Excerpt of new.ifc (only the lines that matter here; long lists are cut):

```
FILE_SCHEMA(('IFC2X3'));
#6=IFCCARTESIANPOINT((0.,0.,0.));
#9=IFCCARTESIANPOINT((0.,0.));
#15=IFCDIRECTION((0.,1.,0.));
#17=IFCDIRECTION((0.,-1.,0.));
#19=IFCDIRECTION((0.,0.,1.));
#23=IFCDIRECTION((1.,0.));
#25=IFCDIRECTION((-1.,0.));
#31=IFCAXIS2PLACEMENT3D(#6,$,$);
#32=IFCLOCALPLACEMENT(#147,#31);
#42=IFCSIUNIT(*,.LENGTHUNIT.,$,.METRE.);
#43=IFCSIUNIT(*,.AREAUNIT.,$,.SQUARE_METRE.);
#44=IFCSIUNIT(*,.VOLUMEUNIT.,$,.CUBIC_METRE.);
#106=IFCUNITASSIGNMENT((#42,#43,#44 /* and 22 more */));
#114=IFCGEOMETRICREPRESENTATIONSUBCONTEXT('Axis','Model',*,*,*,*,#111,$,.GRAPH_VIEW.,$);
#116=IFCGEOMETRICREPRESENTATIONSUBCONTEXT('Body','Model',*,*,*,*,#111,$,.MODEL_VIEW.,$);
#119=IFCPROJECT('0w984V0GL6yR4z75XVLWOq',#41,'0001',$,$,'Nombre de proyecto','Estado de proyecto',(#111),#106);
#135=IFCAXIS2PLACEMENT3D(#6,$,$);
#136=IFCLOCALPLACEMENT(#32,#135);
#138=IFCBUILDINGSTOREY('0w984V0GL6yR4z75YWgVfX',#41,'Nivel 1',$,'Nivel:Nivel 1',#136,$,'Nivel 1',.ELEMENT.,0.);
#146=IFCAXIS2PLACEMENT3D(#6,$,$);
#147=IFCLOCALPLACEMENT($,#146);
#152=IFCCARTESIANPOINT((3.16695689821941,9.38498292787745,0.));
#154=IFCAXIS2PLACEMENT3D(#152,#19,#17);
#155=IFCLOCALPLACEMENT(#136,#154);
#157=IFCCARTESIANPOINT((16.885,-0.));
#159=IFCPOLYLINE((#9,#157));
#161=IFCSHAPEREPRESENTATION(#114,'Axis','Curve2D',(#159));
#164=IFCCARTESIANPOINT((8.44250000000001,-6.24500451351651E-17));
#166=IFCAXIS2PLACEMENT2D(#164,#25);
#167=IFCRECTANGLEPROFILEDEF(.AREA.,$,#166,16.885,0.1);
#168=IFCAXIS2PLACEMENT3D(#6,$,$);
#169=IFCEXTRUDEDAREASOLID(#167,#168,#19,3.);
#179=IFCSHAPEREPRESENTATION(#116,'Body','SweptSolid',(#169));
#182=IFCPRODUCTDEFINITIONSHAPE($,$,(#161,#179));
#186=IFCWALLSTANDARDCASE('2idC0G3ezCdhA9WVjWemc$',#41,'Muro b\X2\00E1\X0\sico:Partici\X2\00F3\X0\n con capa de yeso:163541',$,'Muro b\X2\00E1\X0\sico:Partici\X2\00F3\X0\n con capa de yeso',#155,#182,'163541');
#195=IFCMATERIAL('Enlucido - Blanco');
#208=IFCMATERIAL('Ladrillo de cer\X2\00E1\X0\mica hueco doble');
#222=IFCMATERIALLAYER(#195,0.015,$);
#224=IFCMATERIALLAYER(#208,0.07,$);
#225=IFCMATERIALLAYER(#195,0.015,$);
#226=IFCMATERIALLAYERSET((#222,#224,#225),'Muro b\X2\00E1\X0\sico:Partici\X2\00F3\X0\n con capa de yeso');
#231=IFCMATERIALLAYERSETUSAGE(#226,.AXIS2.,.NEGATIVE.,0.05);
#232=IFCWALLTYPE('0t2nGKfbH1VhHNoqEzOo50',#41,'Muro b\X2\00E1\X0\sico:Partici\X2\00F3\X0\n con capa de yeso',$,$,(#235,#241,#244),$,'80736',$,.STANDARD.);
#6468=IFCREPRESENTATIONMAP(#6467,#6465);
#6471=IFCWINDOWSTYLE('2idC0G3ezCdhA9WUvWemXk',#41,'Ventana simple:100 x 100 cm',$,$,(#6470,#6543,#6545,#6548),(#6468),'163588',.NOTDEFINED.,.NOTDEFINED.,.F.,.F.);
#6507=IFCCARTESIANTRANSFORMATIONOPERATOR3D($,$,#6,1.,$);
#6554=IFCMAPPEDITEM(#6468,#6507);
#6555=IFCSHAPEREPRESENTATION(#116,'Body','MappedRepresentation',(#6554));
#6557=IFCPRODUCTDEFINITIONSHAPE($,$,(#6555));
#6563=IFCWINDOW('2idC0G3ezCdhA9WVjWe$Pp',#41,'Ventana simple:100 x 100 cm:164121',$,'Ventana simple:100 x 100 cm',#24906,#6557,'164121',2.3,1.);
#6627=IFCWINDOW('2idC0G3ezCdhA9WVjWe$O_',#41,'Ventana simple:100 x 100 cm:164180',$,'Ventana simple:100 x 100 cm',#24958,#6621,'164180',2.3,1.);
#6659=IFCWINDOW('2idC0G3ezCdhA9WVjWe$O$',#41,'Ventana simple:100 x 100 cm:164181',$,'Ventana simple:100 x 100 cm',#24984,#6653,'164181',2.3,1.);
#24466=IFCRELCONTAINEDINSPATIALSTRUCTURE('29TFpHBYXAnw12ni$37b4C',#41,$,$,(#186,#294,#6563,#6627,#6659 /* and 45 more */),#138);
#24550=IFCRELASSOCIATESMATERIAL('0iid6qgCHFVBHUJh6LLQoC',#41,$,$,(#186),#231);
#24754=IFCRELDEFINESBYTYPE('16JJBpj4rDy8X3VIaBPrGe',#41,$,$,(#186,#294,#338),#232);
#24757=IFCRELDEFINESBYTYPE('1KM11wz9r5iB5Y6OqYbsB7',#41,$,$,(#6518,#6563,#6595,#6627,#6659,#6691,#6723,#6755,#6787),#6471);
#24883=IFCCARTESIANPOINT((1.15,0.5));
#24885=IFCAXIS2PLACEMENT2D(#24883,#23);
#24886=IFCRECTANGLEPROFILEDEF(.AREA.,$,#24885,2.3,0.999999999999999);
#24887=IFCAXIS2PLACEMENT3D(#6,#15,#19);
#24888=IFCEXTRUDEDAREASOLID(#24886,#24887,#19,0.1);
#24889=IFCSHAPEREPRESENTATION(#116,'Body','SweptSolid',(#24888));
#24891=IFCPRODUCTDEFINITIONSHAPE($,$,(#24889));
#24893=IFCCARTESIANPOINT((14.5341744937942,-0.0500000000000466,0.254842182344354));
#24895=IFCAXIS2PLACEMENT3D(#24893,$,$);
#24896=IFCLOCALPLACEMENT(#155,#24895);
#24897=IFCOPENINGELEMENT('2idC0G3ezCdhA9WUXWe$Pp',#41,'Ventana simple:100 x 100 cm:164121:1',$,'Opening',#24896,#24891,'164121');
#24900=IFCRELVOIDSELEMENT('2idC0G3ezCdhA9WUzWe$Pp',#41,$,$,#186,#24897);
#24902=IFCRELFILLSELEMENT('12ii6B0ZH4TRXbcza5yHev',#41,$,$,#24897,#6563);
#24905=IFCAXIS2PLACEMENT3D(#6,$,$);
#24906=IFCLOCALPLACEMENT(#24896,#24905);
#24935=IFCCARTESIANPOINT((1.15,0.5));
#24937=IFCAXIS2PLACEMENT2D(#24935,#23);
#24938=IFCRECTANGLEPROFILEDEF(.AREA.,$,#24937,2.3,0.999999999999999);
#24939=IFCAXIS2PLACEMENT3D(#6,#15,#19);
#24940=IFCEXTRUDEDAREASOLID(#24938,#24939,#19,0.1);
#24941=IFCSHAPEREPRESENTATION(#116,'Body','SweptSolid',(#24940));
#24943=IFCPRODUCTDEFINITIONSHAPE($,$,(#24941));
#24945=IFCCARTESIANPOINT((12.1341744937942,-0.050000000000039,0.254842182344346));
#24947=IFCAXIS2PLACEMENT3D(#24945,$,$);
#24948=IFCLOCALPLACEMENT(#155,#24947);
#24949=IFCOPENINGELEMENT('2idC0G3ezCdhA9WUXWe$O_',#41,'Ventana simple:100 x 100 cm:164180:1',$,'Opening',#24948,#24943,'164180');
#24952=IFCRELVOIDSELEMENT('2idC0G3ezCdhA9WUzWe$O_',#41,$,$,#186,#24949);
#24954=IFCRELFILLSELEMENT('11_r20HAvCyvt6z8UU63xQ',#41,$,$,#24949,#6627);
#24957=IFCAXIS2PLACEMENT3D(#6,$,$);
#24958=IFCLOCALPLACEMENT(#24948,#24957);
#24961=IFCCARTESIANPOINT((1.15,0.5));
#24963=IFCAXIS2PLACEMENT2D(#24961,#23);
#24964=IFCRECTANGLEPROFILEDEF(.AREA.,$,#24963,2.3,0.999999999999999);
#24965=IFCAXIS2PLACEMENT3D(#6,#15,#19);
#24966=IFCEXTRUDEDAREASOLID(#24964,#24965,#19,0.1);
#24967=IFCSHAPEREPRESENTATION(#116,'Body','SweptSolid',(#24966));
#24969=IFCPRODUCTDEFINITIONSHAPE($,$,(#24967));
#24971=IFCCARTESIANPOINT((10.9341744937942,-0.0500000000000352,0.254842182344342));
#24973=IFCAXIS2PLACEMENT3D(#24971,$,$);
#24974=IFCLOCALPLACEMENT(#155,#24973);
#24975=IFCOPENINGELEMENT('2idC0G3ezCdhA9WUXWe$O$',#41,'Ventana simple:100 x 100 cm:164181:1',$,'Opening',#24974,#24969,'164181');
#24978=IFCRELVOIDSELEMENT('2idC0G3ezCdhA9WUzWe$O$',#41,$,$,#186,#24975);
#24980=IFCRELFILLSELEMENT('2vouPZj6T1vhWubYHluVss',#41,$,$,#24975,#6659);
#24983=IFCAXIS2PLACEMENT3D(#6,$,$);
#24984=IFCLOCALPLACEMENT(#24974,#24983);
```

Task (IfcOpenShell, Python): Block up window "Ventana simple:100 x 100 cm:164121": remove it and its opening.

```python
import ifcopenshell
import ifcopenshell.api.feature
import ifcopenshell.api.root
import ifcopenshell.geom
import ifcopenshell.util.shape

model = ifcopenshell.open("new.ifc")
settings = ifcopenshell.geom.settings()


def volume(element):
    """Net volume in cubic metres, openings subtracted."""
    shape = ifcopenshell.geom.create_shape(settings, element)
    return ifcopenshell.util.shape.get_volume(shape.geometry)


window = model.by_guid("2idC0G3ezCdhA9WVjWe$Pp")
opening = window.FillsVoids[0].RelatingOpeningElement
wall = opening.VoidsElements[0].RelatingBuildingElement
before = volume(wall)

ifcopenshell.api.root.remove_product(model, product=window)
ifcopenshell.api.feature.remove_feature(model, feature=opening)

after = volume(wall)

print(f"wall volume {before:.3f} -> {after:.3f} m3")

model.write("new-out.ifc")
```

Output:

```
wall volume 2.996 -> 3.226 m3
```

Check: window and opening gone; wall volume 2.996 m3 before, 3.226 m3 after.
